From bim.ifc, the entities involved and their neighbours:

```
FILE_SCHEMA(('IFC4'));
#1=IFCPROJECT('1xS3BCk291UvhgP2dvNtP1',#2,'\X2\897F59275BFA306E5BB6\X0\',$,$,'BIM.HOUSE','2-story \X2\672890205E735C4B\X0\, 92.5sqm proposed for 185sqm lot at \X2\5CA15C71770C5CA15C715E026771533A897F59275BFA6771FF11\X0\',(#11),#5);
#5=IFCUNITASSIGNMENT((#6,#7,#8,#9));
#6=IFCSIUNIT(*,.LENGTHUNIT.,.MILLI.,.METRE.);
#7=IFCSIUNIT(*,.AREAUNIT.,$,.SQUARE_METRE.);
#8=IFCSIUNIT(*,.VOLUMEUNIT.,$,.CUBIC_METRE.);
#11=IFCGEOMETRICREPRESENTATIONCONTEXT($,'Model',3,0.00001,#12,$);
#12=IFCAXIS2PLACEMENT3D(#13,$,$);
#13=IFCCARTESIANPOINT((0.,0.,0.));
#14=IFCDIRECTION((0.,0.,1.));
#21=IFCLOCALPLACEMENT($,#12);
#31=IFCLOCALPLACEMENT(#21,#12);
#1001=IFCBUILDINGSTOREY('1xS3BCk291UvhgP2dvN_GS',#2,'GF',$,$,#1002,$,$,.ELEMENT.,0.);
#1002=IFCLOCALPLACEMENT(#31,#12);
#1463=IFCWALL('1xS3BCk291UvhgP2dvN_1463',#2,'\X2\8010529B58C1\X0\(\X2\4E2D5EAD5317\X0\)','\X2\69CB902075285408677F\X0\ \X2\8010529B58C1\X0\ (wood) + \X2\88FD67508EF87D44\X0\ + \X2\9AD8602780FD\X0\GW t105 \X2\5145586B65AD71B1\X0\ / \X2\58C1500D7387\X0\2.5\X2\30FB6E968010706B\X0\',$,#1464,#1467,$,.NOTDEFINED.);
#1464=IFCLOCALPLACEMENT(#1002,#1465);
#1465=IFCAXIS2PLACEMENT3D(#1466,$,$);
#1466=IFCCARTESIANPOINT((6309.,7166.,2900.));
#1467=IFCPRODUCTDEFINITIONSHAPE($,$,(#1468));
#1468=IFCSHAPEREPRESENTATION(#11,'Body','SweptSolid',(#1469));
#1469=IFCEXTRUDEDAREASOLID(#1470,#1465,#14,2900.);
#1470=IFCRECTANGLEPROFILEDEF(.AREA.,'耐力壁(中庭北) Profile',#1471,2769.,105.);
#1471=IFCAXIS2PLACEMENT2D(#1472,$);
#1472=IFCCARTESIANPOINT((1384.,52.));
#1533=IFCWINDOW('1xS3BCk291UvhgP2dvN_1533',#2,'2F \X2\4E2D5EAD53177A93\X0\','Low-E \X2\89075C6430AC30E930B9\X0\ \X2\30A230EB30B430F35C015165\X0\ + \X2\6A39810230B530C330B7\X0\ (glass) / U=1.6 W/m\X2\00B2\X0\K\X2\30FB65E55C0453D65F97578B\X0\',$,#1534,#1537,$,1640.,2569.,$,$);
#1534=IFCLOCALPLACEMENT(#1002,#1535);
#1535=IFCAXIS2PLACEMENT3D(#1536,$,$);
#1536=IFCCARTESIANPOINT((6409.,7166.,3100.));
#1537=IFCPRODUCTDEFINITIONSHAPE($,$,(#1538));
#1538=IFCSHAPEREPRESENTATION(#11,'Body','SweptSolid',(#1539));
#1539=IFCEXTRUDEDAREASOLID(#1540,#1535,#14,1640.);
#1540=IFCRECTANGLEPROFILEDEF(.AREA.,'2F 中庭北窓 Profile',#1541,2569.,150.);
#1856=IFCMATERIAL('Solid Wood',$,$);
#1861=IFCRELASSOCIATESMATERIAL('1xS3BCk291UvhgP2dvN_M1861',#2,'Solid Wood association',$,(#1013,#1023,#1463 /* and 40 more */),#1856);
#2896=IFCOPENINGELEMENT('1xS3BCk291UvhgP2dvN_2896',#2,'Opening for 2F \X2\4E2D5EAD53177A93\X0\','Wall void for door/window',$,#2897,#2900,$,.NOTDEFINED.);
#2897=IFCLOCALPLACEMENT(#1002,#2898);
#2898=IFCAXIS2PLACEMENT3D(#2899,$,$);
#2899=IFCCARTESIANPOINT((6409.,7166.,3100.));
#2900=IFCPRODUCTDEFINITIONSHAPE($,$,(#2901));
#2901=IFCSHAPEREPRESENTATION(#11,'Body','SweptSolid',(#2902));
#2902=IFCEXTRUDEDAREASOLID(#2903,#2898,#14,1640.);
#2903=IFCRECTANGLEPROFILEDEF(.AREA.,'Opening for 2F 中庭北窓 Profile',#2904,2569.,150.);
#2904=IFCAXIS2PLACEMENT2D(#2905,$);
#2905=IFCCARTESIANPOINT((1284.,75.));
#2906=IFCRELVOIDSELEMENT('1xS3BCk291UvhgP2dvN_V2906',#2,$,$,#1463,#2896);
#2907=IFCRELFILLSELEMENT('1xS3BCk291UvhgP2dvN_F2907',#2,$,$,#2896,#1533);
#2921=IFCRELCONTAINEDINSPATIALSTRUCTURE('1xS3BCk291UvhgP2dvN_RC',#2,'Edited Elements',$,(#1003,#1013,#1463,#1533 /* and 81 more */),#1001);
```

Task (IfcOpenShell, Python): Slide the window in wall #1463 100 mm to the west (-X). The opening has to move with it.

```python
import ifcopenshell
import ifcopenshell.api.geometry
import ifcopenshell.util.placement

model = ifcopenshell.open("bim.ifc")

window = model.by_guid("1xS3BCk291UvhgP2dvN_1533")
opening = window.FillsVoids[0].RelatingOpeningElement
wall = opening.VoidsElements[0].RelatingBuildingElement

wall_matrix = ifcopenshell.util.placement.get_local_placement(wall.ObjectPlacement)
shift = wall_matrix[:3, 0] * -100.0
before = ifcopenshell.util.placement.get_local_placement(window.ObjectPlacement)[:3, 3].copy()

# The window is not placed relative to its opening, so move both.
for product in (opening, window):
    matrix = ifcopenshell.util.placement.get_local_placement(product.ObjectPlacement)
    matrix[:3, 3] += shift
    ifcopenshell.api.geometry.edit_object_placement(model, product=product, matrix=matrix, is_si=False)

after = ifcopenshell.util.placement.get_local_placement(window.ObjectPlacement)[:3, 3]
print("window moved by", (after - before).round(3) + 0.0)

model.write("bim-out.ifc")
```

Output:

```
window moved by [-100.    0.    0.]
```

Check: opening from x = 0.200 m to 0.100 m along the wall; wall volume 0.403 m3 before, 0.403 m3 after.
